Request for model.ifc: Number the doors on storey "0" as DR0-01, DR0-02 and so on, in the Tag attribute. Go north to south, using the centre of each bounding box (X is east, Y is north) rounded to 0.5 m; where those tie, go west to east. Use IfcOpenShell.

First a look at what the model holds.

```python
import ifcopenshell
import ifcopenshell.util.element
import ifcopenshell.util.placement

model = ifcopenshell.open("model.ifc")
print(model.schema)
storey = next(s for s in model.by_type("IfcBuildingStorey") if s.Name == "0")
doors = [e for e in ifcopenshell.util.element.get_decomposition(storey) if e.is_a("IfcDoor")]
for e in sorted(doors, key=lambda e: e.id()):
    origin = ifcopenshell.util.placement.get_local_placement(e.ObjectPlacement)[:3, 3]
    print(e.id(), e.Tag, e.Name, origin.round(2) + 0.0, sep=" | ")
```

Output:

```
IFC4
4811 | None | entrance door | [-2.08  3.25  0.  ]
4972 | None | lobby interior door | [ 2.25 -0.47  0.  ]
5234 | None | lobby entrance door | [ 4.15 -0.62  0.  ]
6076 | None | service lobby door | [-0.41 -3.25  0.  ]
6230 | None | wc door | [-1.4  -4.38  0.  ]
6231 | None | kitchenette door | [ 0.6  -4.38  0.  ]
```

```python
import ifcopenshell
import ifcopenshell.geom
import ifcopenshell.util.element
import ifcopenshell.util.shape

model = ifcopenshell.open("model.ifc")
settings = ifcopenshell.geom.settings()
settings.set("use-world-coords", True)


def centre(element):
    shape = ifcopenshell.geom.create_shape(settings, element)
    return ifcopenshell.util.shape.get_bbox_centroid(shape.geometry)


storey = next(s for s in model.by_type("IfcBuildingStorey") if s.Name == "0")
doors = [e for e in ifcopenshell.util.element.get_decomposition(storey) if e.is_a("IfcDoor")]

# Insertion points can sit at a corner or the storey origin, so sort by the geometry (in metres).
centres = {e: centre(e) for e in doors}
doors.sort(key=lambda e: (-round(centres[e][1] / 0.5), centres[e][0]))

for i, e in enumerate(doors, start=1):
    number = f"DR0-{i:02d}"
    e.Tag = number
    print(e.id(), number)

model.write("model_rev.ifc")
```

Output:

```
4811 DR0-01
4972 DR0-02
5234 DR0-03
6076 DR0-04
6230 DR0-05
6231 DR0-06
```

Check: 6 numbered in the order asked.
